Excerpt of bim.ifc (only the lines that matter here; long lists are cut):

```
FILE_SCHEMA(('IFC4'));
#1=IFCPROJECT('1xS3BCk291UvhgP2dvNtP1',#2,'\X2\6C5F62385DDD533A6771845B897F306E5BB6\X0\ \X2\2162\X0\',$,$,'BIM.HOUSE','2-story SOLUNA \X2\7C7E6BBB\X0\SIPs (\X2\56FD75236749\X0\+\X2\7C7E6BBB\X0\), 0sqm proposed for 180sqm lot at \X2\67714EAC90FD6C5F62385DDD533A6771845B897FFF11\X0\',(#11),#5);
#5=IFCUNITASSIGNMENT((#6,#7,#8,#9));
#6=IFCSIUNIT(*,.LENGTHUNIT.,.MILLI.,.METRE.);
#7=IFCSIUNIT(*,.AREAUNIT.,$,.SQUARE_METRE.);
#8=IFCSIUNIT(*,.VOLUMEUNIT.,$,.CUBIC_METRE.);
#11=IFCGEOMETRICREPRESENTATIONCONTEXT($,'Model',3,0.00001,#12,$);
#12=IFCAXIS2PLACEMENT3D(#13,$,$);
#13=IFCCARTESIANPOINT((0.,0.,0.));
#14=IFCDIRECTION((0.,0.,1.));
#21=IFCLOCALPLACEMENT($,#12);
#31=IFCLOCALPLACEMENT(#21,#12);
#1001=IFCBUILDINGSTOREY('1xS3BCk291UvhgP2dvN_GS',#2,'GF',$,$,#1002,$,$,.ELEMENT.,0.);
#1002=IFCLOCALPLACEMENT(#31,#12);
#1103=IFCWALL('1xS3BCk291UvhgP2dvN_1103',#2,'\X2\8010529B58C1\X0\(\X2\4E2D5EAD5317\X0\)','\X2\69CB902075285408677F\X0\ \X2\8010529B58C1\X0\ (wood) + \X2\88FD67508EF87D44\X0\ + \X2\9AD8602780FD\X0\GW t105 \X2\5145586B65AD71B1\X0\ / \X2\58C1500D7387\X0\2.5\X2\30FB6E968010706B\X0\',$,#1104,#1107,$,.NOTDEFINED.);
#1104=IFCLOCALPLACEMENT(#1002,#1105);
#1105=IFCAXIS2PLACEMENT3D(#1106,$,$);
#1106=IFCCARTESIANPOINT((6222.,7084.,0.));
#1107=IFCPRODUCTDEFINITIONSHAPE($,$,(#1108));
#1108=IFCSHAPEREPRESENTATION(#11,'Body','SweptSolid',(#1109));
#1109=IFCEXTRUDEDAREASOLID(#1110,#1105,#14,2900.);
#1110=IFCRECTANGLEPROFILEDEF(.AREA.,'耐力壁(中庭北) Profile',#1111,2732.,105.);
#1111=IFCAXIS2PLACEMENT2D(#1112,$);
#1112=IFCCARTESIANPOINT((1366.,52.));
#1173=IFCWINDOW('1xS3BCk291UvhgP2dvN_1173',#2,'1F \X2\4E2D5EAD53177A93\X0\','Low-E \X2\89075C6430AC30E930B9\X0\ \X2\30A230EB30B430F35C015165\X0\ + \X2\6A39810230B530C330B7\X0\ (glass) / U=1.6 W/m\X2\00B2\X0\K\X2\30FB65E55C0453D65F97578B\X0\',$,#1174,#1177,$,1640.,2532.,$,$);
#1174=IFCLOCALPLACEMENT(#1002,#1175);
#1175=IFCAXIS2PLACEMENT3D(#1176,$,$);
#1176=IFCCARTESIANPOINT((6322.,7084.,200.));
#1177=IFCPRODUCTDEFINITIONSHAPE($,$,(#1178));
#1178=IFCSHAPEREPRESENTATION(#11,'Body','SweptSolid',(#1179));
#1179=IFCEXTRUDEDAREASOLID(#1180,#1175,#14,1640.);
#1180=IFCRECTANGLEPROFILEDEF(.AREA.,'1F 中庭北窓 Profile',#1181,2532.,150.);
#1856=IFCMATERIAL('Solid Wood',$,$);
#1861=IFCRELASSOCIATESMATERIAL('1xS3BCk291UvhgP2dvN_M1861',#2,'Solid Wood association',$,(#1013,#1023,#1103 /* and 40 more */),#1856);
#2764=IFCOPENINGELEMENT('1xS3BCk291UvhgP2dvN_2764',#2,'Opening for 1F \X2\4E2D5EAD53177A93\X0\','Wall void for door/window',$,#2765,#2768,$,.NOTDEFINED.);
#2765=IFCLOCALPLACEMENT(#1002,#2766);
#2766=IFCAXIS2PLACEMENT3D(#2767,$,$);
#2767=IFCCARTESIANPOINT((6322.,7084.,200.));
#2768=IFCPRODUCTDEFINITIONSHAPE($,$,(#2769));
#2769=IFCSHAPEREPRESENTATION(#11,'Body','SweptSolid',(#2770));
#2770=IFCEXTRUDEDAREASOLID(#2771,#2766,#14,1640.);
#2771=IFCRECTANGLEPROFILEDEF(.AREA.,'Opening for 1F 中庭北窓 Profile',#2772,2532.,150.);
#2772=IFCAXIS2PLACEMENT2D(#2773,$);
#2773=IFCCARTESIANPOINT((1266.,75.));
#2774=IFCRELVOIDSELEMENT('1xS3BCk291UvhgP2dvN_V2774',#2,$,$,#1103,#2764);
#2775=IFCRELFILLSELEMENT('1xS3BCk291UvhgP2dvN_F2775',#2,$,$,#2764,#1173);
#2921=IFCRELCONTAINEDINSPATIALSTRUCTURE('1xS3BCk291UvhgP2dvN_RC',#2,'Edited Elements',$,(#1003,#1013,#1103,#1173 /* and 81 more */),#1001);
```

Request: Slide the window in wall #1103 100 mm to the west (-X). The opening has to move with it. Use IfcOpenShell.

```python
import ifcopenshell
import ifcopenshell.api.geometry
import ifcopenshell.util.placement

model = ifcopenshell.open("bim.ifc")

window = model.by_guid("1xS3BCk291UvhgP2dvN_1173")
opening = window.FillsVoids[0].RelatingOpeningElement
wall = opening.VoidsElements[0].RelatingBuildingElement

wall_matrix = ifcopenshell.util.placement.get_local_placement(wall.ObjectPlacement)
shift = wall_matrix[:3, 0] * -100.0
before = ifcopenshell.util.placement.get_local_placement(window.ObjectPlacement)[:3, 3].copy()

# The window is not placed relative to its opening, so move both.
for product in (opening, window):
    matrix = ifcopenshell.util.placement.get_local_placement(product.ObjectPlacement)
    matrix[:3, 3] += shift
    ifcopenshell.api.geometry.edit_object_placement(model, product=product, matrix=matrix, is_si=False)

after = ifcopenshell.util.placement.get_local_placement(window.ObjectPlacement)[:3, 3]
print("window moved by", (after - before).round(3) + 0.0)

model.write("bim-out.ifc")
```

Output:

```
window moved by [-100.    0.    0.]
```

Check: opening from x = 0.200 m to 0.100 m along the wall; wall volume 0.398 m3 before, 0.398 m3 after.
